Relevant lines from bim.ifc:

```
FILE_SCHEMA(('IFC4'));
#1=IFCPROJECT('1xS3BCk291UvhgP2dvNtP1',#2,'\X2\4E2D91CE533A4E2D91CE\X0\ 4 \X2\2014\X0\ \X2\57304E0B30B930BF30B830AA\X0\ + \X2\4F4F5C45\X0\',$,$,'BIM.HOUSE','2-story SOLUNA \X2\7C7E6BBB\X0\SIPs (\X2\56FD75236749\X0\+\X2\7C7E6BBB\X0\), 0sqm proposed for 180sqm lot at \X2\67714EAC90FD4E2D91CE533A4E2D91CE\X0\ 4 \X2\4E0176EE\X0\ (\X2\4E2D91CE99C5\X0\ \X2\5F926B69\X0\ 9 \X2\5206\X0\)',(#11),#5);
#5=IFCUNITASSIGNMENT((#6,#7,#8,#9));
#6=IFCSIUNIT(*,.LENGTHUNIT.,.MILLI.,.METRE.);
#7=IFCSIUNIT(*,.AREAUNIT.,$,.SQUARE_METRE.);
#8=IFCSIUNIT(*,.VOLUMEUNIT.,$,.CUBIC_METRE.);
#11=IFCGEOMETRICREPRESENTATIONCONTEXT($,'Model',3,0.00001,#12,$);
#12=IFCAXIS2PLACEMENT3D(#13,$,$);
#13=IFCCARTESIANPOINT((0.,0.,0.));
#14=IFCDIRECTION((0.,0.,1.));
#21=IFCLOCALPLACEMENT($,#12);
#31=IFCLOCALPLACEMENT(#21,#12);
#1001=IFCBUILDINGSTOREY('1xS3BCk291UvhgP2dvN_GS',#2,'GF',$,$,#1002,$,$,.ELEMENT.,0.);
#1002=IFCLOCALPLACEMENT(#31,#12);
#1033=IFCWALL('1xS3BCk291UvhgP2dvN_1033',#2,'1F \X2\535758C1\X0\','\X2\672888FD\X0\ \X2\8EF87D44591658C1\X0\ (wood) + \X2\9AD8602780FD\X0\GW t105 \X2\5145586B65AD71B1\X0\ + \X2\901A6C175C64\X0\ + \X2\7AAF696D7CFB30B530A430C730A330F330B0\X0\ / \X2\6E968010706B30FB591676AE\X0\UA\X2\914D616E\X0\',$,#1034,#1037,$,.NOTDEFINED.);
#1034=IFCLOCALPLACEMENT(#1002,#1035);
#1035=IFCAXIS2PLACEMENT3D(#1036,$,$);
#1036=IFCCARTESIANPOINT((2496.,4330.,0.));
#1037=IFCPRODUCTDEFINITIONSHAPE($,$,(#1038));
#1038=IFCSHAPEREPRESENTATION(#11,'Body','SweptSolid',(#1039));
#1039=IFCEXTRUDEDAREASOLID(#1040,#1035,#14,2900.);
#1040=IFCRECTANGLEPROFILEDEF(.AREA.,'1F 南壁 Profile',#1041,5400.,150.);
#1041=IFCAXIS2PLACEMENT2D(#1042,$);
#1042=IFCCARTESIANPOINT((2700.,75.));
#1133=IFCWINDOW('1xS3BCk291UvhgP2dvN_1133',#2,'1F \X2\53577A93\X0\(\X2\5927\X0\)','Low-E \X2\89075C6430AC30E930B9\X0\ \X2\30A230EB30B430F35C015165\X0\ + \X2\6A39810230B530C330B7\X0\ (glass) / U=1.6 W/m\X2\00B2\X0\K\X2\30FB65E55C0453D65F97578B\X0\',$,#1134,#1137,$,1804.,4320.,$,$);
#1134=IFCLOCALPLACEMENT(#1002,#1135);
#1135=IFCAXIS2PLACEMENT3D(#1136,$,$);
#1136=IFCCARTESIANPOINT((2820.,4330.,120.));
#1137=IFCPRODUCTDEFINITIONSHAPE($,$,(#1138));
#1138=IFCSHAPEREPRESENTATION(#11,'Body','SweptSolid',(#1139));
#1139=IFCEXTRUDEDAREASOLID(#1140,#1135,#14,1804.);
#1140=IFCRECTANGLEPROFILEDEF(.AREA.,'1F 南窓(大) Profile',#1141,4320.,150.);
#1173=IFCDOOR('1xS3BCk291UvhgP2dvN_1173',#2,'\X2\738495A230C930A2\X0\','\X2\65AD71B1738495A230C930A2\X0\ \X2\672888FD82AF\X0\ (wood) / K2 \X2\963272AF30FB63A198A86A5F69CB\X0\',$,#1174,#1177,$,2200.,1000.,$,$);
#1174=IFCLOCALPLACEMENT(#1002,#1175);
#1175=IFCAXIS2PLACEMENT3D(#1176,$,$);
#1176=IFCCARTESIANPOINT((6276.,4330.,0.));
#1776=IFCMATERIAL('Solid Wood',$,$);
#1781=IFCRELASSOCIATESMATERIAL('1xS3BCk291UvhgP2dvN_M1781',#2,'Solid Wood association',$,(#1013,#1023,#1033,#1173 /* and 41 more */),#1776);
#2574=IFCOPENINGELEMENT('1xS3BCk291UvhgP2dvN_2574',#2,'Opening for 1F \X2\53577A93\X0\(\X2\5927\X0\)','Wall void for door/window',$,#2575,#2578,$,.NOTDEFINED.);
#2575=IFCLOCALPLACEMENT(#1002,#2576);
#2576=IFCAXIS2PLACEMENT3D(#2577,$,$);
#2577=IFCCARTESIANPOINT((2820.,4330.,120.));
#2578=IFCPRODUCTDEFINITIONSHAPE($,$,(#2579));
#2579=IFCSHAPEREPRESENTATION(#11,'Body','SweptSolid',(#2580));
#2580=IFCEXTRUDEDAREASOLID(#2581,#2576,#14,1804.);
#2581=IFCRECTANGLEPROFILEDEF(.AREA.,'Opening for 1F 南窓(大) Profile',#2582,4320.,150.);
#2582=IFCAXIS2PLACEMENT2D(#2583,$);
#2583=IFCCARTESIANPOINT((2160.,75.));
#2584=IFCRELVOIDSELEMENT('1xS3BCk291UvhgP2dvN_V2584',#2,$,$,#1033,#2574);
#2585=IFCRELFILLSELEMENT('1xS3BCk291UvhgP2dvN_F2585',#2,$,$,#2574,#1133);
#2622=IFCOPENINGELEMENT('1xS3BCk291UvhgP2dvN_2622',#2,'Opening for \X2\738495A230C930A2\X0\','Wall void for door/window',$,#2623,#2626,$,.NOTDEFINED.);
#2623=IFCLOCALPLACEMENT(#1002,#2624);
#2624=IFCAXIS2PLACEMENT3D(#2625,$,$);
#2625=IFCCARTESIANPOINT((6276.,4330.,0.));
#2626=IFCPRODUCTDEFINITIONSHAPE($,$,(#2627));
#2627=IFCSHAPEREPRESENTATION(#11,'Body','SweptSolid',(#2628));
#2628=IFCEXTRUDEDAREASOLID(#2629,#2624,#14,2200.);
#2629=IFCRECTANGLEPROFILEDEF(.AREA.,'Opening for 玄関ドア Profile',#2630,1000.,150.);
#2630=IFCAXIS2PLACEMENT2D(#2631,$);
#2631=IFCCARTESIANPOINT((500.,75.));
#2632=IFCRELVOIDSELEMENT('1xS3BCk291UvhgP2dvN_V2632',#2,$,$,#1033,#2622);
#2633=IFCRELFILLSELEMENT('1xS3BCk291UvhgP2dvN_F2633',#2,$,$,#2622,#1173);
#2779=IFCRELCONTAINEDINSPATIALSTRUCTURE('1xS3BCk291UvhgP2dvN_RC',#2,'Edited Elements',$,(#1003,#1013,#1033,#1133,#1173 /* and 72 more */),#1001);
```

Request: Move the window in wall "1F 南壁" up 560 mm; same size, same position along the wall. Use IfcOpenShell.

```python
import numpy as np
import ifcopenshell
import ifcopenshell.api.geometry
import ifcopenshell.util.placement
import ifcopenshell.util.unit

model = ifcopenshell.open("bim.ifc")
unit_scale = ifcopenshell.util.unit.calculate_unit_scale(model)

window = model.by_guid("1xS3BCk291UvhgP2dvN_1133")
opening = window.FillsVoids[0].RelatingOpeningElement
dz = 560.0

shift = np.array([0.0, 0.0, dz])
# The window is not placed relative to its opening, so move both.
for product in (opening, window):
    matrix = ifcopenshell.util.placement.get_local_placement(product.ObjectPlacement)
    matrix[:3, 3] += shift
    ifcopenshell.api.geometry.edit_object_placement(model, product=product, matrix=matrix, is_si=False)

print(f"moved by {dz * unit_scale:+.3f} m")

model.write("bim_v2.ifc")
```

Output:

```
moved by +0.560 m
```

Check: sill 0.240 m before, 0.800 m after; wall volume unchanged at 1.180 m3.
